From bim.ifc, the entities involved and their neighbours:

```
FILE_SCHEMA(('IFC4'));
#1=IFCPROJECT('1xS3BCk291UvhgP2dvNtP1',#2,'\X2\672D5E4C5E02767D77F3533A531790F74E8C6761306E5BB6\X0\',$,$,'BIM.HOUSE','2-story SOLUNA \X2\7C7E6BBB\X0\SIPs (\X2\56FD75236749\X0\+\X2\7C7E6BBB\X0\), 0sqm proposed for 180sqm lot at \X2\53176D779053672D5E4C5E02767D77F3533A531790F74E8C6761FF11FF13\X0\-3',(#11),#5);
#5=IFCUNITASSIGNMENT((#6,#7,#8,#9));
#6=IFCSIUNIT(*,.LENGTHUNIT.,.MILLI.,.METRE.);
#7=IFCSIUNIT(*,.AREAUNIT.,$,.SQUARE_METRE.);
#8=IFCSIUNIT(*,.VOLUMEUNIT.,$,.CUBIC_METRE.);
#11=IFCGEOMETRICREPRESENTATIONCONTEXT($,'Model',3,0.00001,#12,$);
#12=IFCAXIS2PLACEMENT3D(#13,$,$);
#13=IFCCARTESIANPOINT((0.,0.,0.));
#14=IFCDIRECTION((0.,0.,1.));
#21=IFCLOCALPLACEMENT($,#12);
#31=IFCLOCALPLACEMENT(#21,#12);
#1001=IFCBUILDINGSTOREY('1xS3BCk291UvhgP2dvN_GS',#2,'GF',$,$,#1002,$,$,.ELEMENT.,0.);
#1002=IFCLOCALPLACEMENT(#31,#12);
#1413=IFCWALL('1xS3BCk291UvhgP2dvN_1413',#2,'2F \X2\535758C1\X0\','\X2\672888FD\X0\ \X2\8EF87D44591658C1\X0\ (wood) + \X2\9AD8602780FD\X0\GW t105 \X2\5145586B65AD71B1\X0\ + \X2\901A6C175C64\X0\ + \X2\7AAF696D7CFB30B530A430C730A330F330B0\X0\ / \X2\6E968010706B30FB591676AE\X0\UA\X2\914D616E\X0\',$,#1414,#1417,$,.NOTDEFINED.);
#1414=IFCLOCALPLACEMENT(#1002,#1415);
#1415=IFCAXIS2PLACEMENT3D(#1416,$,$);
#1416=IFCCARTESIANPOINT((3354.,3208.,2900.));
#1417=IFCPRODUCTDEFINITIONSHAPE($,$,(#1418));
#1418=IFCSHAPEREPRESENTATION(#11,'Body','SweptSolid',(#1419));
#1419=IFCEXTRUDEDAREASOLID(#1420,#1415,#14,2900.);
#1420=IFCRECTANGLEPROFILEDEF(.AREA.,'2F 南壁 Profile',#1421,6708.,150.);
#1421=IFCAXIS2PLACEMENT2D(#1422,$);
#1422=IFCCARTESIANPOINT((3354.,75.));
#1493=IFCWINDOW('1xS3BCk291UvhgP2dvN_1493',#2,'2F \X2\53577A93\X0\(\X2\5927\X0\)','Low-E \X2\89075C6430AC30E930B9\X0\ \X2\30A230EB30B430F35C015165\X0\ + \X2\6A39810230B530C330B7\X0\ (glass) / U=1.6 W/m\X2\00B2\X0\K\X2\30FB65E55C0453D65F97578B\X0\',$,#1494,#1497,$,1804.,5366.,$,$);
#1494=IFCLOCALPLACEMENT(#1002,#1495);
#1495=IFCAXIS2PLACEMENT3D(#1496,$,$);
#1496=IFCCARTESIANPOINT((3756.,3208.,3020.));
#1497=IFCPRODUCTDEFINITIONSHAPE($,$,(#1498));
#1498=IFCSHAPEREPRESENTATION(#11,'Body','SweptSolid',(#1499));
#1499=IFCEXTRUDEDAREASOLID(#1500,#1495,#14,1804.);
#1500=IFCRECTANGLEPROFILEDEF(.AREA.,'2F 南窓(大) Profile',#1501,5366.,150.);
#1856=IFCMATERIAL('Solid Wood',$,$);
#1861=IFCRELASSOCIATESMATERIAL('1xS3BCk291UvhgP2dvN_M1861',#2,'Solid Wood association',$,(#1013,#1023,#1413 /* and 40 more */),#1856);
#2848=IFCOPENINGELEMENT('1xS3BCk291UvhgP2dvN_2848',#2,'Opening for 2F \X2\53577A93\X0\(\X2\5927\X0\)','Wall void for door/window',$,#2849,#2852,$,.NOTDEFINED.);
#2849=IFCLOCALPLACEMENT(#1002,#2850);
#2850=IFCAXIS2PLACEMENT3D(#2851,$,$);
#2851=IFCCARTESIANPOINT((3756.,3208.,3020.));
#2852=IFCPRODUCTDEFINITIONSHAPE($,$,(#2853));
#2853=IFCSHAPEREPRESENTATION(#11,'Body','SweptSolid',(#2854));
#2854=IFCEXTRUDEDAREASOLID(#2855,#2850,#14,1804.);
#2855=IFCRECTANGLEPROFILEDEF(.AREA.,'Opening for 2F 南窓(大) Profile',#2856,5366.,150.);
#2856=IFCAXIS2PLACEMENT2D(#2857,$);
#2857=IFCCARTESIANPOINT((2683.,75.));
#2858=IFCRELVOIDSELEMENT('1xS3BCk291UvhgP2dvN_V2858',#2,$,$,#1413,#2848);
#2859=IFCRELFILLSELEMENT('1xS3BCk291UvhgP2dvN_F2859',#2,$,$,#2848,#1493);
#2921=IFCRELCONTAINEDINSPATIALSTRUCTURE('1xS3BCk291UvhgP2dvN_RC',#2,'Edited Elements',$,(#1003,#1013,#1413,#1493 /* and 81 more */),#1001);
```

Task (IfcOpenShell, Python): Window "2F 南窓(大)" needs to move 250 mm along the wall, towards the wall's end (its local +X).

```python
import ifcopenshell
import ifcopenshell.api.geometry
import ifcopenshell.util.placement
import ifcopenshell.util.unit

model = ifcopenshell.open("bim.ifc")
unit_scale = ifcopenshell.util.unit.calculate_unit_scale(model)

window = model.by_id(1493)
opening = window.FillsVoids[0].RelatingOpeningElement
wall = opening.VoidsElements[0].RelatingBuildingElement

wall_matrix = ifcopenshell.util.placement.get_local_placement(wall.ObjectPlacement)
shift = wall_matrix[:3, 0] * 0.25 / unit_scale
before = ifcopenshell.util.placement.get_local_placement(window.ObjectPlacement)[:3, 3].copy()

# The window is not placed relative to its opening, so move both.
for product in (opening, window):
    matrix = ifcopenshell.util.placement.get_local_placement(product.ObjectPlacement)
    matrix[:3, 3] += shift
    ifcopenshell.api.geometry.edit_object_placement(model, product=product, matrix=matrix, is_si=False)

after = ifcopenshell.util.placement.get_local_placement(window.ObjectPlacement)[:3, 3]
print("window moved by", (after - before).round(3) + 0.0)

model.write("bim-out.ifc")
```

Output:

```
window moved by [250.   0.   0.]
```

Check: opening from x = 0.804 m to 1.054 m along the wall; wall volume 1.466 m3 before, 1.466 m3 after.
